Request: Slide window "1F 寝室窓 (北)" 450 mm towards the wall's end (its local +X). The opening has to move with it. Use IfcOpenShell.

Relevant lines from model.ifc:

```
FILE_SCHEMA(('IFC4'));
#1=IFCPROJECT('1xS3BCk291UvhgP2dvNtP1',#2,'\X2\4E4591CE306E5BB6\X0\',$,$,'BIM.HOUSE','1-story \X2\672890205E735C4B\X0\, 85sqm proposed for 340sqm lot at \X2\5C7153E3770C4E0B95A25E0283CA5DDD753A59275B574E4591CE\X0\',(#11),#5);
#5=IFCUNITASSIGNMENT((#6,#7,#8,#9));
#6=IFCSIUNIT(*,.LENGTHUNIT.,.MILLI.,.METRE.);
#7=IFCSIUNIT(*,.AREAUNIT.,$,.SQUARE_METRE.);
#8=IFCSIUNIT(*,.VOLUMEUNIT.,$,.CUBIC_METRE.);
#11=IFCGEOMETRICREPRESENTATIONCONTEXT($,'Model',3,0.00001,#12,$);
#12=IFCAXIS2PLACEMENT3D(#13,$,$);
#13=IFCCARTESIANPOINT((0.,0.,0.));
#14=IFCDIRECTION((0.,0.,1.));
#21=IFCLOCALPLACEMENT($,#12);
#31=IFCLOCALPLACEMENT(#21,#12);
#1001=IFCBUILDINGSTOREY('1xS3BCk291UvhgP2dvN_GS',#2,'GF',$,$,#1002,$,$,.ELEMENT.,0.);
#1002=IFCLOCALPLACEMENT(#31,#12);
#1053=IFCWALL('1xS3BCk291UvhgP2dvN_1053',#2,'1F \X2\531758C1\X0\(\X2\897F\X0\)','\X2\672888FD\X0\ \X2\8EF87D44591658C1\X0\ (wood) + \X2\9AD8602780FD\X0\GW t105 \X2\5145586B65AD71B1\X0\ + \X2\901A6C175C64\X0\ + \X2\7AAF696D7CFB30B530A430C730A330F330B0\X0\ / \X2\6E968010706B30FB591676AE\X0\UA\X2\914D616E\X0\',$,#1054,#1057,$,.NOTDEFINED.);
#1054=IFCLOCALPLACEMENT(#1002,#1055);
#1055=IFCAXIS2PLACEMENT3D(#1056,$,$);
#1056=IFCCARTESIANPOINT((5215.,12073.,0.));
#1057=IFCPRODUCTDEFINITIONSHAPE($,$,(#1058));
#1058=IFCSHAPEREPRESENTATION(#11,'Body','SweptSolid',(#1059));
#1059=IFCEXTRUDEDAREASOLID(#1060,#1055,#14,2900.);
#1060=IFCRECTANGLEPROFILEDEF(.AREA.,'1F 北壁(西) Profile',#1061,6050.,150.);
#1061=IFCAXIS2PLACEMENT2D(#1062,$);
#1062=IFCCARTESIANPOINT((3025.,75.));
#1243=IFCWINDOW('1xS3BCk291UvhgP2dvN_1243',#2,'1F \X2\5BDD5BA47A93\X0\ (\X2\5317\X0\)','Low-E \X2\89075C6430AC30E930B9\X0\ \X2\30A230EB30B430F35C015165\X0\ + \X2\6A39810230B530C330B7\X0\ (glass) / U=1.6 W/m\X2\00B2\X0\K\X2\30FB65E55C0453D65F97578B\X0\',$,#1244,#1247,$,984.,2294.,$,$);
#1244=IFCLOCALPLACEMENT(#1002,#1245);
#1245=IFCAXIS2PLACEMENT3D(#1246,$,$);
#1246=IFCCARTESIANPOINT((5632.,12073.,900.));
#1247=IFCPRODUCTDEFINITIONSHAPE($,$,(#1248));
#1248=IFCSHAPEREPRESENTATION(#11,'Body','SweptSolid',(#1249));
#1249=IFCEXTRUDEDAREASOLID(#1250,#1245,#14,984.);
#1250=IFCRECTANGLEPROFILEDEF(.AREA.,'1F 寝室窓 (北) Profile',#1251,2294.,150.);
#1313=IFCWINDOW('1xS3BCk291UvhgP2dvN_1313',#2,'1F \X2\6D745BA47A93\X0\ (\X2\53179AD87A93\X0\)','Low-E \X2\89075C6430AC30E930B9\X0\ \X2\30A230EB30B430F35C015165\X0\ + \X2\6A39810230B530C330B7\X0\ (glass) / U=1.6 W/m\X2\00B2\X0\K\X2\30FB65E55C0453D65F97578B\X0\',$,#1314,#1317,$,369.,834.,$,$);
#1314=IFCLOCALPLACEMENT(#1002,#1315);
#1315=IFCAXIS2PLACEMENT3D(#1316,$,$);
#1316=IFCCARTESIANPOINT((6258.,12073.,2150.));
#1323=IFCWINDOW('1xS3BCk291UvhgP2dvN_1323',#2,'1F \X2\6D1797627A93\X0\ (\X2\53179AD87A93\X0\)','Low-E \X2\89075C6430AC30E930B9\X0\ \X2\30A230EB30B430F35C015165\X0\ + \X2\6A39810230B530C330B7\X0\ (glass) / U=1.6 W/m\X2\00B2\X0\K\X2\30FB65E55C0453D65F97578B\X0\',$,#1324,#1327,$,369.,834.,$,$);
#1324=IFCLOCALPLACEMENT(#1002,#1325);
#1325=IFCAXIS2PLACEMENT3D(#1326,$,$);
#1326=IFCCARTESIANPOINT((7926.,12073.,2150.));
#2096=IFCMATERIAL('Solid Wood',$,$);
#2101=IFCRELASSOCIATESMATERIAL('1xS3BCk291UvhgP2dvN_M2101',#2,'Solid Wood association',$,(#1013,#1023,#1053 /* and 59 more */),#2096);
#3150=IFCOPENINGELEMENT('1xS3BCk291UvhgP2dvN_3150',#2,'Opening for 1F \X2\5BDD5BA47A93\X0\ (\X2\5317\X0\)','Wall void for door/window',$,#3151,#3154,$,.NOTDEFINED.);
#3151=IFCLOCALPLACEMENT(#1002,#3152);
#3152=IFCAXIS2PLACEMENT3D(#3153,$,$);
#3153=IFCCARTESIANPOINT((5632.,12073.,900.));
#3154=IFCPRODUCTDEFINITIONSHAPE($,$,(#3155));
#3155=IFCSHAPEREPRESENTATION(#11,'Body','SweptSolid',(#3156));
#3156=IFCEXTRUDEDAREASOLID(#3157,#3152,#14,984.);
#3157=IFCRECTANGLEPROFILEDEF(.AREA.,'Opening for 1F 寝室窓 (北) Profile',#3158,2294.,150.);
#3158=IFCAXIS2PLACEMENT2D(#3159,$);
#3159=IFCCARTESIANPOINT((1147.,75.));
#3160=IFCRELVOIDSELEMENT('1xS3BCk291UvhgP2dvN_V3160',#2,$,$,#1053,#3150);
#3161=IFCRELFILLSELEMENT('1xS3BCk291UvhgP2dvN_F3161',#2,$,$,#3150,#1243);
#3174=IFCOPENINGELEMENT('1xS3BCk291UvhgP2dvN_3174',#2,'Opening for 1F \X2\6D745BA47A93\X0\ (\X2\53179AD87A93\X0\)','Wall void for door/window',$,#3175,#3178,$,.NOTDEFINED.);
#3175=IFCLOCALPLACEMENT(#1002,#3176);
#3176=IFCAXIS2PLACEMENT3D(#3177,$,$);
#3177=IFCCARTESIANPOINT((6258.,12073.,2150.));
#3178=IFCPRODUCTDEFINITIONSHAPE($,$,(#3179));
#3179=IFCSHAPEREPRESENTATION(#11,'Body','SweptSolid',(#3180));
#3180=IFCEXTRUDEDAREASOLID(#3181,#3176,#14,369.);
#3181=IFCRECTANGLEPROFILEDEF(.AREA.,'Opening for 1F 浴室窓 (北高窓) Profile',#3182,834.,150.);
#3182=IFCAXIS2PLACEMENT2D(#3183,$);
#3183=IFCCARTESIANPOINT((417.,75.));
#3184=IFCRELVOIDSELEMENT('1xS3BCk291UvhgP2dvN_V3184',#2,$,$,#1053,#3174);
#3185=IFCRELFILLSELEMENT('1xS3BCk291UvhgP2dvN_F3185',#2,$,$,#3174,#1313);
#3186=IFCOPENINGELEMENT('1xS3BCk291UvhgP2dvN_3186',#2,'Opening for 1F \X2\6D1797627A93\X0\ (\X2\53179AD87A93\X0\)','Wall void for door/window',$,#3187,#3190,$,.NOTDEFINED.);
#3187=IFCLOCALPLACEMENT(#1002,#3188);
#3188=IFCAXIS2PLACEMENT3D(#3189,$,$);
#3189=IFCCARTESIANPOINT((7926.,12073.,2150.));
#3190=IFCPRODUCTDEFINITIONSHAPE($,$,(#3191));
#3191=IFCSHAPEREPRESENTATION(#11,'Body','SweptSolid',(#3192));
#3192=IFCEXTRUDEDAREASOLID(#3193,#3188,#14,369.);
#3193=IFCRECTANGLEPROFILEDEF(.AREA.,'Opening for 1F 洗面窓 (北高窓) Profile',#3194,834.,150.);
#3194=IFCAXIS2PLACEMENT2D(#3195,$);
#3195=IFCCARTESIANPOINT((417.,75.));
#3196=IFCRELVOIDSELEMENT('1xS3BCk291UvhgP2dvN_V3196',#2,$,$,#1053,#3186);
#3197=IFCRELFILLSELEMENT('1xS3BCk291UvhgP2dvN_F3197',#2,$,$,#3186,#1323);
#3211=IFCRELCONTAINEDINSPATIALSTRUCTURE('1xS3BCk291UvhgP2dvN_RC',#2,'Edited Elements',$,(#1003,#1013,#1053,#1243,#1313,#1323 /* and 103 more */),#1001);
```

```python
import ifcopenshell
import ifcopenshell.api.geometry
import ifcopenshell.util.placement
import ifcopenshell.util.unit

model = ifcopenshell.open("model.ifc")
unit_scale = ifcopenshell.util.unit.calculate_unit_scale(model)

window = model.by_guid("1xS3BCk291UvhgP2dvN_1243")
opening = window.FillsVoids[0].RelatingOpeningElement
wall = opening.VoidsElements[0].RelatingBuildingElement

wall_matrix = ifcopenshell.util.placement.get_local_placement(wall.ObjectPlacement)
shift = wall_matrix[:3, 0] * 0.45 / unit_scale
before = ifcopenshell.util.placement.get_local_placement(window.ObjectPlacement)[:3, 3].copy()

# The window is not placed relative to its opening, so move both.
for product in (opening, window):
    matrix = ifcopenshell.util.placement.get_local_placement(product.ObjectPlacement)
    matrix[:3, 3] += shift
    ifcopenshell.api.geometry.edit_object_placement(model, product=product, matrix=matrix, is_si=False)

after = ifcopenshell.util.placement.get_local_placement(window.ObjectPlacement)[:3, 3]
print("window moved by", (after - before).round(3) + 0.0)

model.write("model-out.ifc")
```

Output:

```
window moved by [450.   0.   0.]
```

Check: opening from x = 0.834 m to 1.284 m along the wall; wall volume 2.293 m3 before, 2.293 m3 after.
